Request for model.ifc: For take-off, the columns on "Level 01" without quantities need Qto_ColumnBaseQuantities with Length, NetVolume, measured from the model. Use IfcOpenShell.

First a look at what the model holds.

```python
import ifcopenshell
import ifcopenshell.util.element
import ifcopenshell.util.unit

model = ifcopenshell.open("model.ifc")
print(model.schema)
for unit_type in ("LENGTHUNIT", "AREAUNIT", "VOLUMEUNIT"):
    print(unit_type, ifcopenshell.util.unit.calculate_unit_scale(model, unit_type))
storey = next(s for s in model.by_type("IfcBuildingStorey") if s.Name == "Level 01")
columns = [e for e in ifcopenshell.util.element.get_decomposition(storey) if e.is_a("IfcColumn")]
for e in sorted(columns, key=lambda e: e.id()):
    print(e.id(), e.is_a(), e.Name, list(ifcopenshell.util.element.get_psets(e, qtos_only=True)), sep=" | ")
```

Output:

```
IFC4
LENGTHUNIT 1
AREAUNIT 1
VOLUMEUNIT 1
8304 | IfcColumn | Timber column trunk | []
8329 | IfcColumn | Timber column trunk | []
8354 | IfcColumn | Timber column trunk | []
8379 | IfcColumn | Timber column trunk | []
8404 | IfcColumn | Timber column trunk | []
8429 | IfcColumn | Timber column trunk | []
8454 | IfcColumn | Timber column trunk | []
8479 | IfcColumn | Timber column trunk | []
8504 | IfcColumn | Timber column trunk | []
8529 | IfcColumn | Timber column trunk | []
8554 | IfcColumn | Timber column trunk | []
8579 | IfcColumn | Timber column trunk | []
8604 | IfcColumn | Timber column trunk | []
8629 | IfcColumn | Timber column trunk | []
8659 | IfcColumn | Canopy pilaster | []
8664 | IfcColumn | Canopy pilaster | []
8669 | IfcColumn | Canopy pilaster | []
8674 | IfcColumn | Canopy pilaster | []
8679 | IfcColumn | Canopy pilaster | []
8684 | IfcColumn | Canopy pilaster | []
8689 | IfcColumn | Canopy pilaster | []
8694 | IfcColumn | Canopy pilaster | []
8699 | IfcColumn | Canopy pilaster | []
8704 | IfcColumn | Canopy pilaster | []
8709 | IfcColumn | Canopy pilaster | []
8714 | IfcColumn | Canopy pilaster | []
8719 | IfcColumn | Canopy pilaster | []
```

```python
import ifcopenshell
import ifcopenshell.api.pset
import ifcopenshell.geom
import ifcopenshell.util.element
import ifcopenshell.util.shape
import ifcopenshell.util.unit

model = ifcopenshell.open("model.ifc")
unit_scale = ifcopenshell.util.unit.calculate_unit_scale(model)
volume_scale = ifcopenshell.util.unit.calculate_unit_scale(model, "VOLUMEUNIT")
settings = ifcopenshell.geom.settings()

storey = next(s for s in model.by_type("IfcBuildingStorey") if s.Name == "Level 01")
columns = [e for e in ifcopenshell.util.element.get_decomposition(storey) if e.is_a("IfcColumn")]

for e in sorted(columns, key=lambda e: e.id()):
    if ifcopenshell.util.element.get_psets(e, qtos_only=True, should_inherit=False):
        continue
    # Geometry comes back in metres, in the element's own axes.
    shape = ifcopenshell.geom.create_shape(settings, e)
    values = {
        "Length": ifcopenshell.util.shape.get_z(shape.geometry) / unit_scale,
        "NetVolume": ifcopenshell.util.shape.get_volume(shape.geometry) / volume_scale,
    }
    qto = ifcopenshell.api.pset.add_qto(model, product=e, name="Qto_ColumnBaseQuantities")
    ifcopenshell.api.pset.edit_qto(model, qto=qto, properties=values)
    print(e.id(), {k: round(v, 3) for k, v in values.items()})

model.write("model-out.ifc")
```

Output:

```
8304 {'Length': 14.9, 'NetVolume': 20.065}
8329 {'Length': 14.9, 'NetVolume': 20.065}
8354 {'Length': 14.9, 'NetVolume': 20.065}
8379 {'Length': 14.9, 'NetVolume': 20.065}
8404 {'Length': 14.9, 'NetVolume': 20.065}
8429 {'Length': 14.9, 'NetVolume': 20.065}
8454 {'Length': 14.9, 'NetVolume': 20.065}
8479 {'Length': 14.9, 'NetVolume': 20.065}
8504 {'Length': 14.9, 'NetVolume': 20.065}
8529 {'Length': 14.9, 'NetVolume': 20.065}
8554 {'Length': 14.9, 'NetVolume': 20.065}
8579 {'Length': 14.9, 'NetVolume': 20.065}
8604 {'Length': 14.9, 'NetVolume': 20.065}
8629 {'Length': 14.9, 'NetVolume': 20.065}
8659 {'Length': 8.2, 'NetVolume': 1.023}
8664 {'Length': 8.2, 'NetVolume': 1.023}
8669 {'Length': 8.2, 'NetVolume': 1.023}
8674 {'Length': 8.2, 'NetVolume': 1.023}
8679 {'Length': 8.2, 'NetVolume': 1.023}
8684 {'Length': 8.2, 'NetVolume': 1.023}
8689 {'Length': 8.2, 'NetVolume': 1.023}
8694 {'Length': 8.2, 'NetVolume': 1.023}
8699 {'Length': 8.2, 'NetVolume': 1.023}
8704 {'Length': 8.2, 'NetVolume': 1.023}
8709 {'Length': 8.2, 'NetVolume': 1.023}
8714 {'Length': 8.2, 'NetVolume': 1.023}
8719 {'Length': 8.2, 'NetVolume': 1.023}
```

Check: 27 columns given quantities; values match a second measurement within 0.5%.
